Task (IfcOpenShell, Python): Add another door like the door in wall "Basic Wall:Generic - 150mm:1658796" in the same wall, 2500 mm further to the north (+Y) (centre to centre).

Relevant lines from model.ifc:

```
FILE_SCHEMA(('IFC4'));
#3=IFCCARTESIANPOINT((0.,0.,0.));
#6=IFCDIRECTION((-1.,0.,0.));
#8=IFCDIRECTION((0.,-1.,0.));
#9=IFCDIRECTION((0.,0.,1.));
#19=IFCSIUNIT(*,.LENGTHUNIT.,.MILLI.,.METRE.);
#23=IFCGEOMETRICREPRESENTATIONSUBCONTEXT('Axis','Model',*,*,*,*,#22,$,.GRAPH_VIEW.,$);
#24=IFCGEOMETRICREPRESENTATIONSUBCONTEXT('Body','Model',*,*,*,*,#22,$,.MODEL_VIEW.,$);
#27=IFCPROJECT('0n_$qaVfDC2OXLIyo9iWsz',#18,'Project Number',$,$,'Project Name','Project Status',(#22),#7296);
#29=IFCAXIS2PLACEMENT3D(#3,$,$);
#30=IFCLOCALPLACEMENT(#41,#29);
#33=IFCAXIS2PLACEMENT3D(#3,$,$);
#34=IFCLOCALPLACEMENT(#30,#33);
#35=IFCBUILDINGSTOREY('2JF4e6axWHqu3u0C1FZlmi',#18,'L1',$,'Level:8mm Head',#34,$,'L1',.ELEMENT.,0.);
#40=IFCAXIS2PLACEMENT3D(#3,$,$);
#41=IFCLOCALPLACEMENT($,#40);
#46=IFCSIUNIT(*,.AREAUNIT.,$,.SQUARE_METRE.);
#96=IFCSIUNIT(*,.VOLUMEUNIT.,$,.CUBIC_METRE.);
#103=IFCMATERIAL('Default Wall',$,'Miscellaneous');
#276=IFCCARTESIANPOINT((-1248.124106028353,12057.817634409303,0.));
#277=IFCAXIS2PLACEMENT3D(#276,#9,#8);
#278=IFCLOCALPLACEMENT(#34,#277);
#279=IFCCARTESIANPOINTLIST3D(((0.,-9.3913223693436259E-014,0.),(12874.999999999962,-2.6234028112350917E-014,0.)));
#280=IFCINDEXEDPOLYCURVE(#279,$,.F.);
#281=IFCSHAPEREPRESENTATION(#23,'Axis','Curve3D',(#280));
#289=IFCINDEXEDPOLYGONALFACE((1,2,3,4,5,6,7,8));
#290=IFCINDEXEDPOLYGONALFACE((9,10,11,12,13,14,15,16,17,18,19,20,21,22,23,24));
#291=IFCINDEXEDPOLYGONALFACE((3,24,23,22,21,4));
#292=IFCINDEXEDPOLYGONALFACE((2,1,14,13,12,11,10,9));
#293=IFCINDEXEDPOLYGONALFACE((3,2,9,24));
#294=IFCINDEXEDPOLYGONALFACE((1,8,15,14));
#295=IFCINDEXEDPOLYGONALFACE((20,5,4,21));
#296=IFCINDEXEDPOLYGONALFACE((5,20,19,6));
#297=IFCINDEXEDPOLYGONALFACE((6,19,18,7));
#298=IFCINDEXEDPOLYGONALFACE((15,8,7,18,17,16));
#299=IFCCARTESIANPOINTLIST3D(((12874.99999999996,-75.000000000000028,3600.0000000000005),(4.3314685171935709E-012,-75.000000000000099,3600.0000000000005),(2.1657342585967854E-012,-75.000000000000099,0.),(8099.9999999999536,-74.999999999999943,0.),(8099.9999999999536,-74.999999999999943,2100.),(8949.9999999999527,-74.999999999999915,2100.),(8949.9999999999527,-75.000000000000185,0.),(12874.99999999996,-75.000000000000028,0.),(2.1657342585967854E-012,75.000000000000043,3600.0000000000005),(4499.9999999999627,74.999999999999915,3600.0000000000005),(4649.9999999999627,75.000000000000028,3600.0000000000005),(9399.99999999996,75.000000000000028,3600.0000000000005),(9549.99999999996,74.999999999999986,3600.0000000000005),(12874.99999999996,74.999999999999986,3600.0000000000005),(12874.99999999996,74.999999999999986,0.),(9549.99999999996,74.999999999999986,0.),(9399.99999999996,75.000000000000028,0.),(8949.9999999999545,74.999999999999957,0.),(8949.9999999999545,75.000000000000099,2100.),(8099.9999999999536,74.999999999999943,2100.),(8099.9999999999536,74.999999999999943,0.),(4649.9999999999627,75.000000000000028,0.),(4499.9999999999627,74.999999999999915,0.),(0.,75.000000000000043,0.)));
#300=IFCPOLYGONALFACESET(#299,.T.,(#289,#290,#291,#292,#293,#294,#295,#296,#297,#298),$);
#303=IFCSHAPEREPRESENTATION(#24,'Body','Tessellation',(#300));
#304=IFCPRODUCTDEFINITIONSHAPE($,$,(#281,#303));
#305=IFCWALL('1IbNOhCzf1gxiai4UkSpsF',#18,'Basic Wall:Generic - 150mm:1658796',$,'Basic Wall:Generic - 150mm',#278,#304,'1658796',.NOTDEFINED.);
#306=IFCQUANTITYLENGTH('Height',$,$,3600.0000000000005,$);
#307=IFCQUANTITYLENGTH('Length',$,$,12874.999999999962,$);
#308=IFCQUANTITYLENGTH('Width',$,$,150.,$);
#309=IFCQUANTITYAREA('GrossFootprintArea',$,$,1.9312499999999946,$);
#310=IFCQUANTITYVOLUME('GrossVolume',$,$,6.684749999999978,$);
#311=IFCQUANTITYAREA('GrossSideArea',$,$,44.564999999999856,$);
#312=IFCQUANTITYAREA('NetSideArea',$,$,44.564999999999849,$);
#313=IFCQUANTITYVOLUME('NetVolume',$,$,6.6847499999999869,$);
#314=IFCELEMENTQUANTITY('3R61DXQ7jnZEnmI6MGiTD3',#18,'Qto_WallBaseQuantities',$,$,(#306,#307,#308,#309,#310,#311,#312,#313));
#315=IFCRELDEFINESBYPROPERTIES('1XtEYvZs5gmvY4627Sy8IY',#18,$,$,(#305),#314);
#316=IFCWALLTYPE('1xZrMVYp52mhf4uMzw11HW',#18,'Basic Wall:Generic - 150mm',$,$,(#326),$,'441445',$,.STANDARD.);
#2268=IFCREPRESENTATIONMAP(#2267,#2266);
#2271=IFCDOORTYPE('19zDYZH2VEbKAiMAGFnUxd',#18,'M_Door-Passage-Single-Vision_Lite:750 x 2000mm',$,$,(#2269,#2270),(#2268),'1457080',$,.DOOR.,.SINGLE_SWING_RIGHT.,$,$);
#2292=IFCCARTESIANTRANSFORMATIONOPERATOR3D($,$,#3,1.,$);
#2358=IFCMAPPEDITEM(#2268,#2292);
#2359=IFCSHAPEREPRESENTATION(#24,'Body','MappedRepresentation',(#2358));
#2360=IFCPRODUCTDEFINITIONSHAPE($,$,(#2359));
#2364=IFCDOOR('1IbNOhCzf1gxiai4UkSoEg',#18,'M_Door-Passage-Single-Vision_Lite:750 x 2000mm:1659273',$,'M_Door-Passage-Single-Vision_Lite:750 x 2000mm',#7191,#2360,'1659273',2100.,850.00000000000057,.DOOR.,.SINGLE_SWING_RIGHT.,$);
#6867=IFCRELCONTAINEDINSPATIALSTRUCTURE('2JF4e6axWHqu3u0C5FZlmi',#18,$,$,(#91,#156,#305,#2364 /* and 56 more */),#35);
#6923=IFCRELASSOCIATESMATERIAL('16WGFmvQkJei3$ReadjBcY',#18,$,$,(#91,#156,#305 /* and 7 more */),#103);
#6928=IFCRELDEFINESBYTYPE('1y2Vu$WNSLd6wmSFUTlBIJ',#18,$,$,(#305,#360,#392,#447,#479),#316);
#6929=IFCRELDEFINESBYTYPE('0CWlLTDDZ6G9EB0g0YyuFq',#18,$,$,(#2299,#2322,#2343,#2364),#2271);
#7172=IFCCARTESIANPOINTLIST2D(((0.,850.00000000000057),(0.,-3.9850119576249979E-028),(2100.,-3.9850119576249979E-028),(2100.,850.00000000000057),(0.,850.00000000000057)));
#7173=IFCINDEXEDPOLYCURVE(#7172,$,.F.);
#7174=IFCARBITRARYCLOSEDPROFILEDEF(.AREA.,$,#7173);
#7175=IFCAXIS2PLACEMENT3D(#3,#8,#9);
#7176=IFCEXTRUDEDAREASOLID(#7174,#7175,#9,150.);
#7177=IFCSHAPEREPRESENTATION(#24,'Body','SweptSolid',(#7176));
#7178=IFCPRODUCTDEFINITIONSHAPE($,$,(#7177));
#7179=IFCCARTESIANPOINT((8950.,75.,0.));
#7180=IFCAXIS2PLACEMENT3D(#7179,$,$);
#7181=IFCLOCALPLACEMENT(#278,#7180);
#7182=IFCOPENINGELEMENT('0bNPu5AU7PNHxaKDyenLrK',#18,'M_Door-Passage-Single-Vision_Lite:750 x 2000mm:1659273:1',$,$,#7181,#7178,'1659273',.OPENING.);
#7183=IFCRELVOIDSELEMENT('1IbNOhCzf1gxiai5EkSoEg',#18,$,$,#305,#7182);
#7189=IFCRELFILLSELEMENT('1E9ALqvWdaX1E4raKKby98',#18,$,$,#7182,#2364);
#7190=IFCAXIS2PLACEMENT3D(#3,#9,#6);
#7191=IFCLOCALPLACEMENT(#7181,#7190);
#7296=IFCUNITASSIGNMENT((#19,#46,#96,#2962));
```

```python
import ifcopenshell
import ifcopenshell.api.feature
import ifcopenshell.api.geometry
import ifcopenshell.api.pset
import ifcopenshell.api.root
import ifcopenshell.geom
import ifcopenshell.util.element
import ifcopenshell.util.placement
import ifcopenshell.util.shape
import ifcopenshell.util.unit

model = ifcopenshell.open("model.ifc")
area_scale = ifcopenshell.util.unit.calculate_unit_scale(model, "AREAUNIT")
volume_scale = ifcopenshell.util.unit.calculate_unit_scale(model, "VOLUMEUNIT")
settings = ifcopenshell.geom.settings()


def volume(element):
    """Net volume in cubic metres, openings subtracted."""
    shape = ifcopenshell.geom.create_shape(settings, element)
    return ifcopenshell.util.shape.get_volume(shape.geometry)


def reuse_history(source, copy):
    """copy_class also copies each property set's owner history, people and application; keep the originals."""
    for rel in copy.IsDefinedBy:
        if rel.is_a("IfcRelDefinesByProperties") and (history := rel.RelatingPropertyDefinition.OwnerHistory):
            rel.RelatingPropertyDefinition.OwnerHistory = source.OwnerHistory
            ifcopenshell.util.element.remove_deep2(model, history)


door = model.by_guid("1IbNOhCzf1gxiai4UkSoEg")
opening = door.FillsVoids[0].RelatingOpeningElement
wall = opening.VoidsElements[0].RelatingBuildingElement
before = volume(wall)
shift = ifcopenshell.util.placement.get_local_placement(wall.ObjectPlacement)[:3, 0] * -2500.0

# copy_class copies the void relationship, type, container and properties, but no geometry.
new_opening = ifcopenshell.api.root.copy_class(model, product=opening)
new_opening.Representation = ifcopenshell.util.element.copy_deep(
    model, opening.Representation, exclude=["IfcGeometricRepresentationContext", "IfcRepresentationMap"]
)
new_opening.Name = "M_Door-Passage-Single-Vision_Lite:750 x 2000mm"
new_opening.Tag = None
reuse_history(opening, new_opening)
new_door = ifcopenshell.api.root.copy_class(model, product=door)
new_door.Representation = ifcopenshell.util.element.copy_deep(
    model, door.Representation, exclude=["IfcGeometricRepresentationContext", "IfcRepresentationMap"]
)
new_door.Name = "M_Door-Passage-Single-Vision_Lite:750 x 2000mm"
new_door.Tag = None
reuse_history(door, new_door)
ifcopenshell.api.feature.add_filling(model, opening=new_opening, element=new_door)

for old, new in ((opening, new_opening), (door, new_door)):
    matrix = ifcopenshell.util.placement.get_local_placement(old.ObjectPlacement)
    matrix[:3, 3] += shift
    ifcopenshell.api.geometry.edit_object_placement(model, product=new, matrix=matrix, is_si=False)

after = volume(wall)
thickness = 0.15  # wall thickness in metres

# Update the wall's stored quantities.
qto = model.by_id(ifcopenshell.util.element.get_pset(wall, "Qto_WallBaseQuantities", should_inherit=False)["id"])
ifcopenshell.api.pset.edit_qto(model, qto=qto, properties={
    "NetSideArea": after / thickness / area_scale,
    "NetVolume": after / volume_scale,
})

print(f"wall volume {before:.3f} -> {after:.3f} m3")

model.write("model-out.ifc")
```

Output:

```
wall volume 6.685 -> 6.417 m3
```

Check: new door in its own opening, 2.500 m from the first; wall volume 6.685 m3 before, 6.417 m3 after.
